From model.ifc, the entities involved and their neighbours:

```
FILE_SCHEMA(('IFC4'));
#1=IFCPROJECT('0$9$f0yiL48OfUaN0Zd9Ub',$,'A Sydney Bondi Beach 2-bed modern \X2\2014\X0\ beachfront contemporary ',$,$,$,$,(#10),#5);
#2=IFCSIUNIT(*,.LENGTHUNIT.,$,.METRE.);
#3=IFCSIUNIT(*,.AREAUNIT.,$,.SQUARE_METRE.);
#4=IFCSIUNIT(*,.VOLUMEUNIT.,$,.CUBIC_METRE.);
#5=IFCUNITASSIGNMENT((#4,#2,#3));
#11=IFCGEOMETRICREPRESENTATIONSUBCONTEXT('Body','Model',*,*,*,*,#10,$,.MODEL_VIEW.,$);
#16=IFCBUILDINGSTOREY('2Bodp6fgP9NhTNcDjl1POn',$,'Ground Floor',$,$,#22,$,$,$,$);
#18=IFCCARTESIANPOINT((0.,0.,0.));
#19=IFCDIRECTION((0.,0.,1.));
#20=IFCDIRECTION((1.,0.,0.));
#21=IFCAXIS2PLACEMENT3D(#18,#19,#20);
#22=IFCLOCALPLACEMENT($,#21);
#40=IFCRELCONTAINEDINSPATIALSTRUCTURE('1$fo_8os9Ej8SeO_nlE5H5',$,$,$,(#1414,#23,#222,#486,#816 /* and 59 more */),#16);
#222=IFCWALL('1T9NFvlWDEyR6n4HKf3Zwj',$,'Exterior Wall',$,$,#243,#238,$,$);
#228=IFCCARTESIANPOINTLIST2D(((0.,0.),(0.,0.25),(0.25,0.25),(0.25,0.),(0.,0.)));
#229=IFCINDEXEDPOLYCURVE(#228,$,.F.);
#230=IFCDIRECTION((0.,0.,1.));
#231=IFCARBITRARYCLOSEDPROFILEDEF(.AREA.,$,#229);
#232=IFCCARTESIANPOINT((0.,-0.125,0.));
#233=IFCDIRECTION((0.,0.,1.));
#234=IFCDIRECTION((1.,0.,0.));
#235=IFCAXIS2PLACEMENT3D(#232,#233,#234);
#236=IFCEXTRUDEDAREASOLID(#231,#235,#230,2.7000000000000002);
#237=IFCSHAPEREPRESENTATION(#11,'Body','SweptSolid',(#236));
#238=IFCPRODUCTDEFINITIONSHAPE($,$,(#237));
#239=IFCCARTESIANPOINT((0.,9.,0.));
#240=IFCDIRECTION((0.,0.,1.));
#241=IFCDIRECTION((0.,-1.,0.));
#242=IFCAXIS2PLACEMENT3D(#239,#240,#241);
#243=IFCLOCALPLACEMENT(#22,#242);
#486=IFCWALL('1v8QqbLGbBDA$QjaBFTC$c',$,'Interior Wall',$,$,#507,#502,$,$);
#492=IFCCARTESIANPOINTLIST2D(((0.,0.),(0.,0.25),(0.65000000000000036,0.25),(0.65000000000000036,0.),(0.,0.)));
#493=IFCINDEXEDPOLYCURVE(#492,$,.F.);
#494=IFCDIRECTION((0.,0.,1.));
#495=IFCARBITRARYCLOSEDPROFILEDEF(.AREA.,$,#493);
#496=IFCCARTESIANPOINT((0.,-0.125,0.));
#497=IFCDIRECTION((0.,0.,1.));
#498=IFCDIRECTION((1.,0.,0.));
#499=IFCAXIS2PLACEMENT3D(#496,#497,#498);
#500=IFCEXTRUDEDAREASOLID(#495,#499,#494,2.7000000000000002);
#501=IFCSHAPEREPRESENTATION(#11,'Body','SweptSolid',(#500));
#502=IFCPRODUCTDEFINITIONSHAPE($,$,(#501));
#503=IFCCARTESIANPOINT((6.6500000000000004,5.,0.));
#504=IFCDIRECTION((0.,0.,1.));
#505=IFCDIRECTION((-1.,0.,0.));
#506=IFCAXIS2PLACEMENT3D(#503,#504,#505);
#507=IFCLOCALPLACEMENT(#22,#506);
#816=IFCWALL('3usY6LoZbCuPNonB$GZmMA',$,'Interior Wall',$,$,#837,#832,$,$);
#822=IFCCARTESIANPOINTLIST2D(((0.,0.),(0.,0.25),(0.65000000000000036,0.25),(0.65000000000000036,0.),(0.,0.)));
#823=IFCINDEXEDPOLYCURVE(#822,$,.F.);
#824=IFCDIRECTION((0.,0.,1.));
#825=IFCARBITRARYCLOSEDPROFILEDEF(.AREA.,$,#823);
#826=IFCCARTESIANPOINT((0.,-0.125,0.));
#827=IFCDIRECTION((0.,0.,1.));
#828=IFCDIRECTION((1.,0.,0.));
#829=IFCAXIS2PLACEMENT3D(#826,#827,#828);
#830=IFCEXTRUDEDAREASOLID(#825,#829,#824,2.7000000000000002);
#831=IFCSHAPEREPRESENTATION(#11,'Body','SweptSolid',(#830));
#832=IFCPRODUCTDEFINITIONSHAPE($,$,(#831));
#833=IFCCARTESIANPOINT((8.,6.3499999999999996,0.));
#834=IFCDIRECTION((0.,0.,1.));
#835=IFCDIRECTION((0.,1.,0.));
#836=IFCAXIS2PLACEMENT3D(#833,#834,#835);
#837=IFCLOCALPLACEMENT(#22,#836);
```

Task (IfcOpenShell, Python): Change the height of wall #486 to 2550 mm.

```python
import ifcopenshell
import ifcopenshell.geom
import ifcopenshell.util.representation
import ifcopenshell.util.shape
import ifcopenshell.util.unit

model = ifcopenshell.open("model.ifc")
unit_scale = ifcopenshell.util.unit.calculate_unit_scale(model)
settings = ifcopenshell.geom.settings()


def volume(element):
    """Net volume in cubic metres, openings subtracted."""
    shape = ifcopenshell.geom.create_shape(settings, element)
    return ifcopenshell.util.shape.get_volume(shape.geometry)


wall = model.by_id(486)
before = volume(wall)

body = ifcopenshell.util.representation.get_representation(wall, "Model", "Body")
solid = body.Items[0]
old_height = solid.Depth
solid.Depth = 2.55 / unit_scale
after = volume(wall)

print(f"height {old_height:g} -> {solid.Depth:g}, volume {before:.3f} -> {after:.3f} m3")

model.write("model_rev.ifc")
```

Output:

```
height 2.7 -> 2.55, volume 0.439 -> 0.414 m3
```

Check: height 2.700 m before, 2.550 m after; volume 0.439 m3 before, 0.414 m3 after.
